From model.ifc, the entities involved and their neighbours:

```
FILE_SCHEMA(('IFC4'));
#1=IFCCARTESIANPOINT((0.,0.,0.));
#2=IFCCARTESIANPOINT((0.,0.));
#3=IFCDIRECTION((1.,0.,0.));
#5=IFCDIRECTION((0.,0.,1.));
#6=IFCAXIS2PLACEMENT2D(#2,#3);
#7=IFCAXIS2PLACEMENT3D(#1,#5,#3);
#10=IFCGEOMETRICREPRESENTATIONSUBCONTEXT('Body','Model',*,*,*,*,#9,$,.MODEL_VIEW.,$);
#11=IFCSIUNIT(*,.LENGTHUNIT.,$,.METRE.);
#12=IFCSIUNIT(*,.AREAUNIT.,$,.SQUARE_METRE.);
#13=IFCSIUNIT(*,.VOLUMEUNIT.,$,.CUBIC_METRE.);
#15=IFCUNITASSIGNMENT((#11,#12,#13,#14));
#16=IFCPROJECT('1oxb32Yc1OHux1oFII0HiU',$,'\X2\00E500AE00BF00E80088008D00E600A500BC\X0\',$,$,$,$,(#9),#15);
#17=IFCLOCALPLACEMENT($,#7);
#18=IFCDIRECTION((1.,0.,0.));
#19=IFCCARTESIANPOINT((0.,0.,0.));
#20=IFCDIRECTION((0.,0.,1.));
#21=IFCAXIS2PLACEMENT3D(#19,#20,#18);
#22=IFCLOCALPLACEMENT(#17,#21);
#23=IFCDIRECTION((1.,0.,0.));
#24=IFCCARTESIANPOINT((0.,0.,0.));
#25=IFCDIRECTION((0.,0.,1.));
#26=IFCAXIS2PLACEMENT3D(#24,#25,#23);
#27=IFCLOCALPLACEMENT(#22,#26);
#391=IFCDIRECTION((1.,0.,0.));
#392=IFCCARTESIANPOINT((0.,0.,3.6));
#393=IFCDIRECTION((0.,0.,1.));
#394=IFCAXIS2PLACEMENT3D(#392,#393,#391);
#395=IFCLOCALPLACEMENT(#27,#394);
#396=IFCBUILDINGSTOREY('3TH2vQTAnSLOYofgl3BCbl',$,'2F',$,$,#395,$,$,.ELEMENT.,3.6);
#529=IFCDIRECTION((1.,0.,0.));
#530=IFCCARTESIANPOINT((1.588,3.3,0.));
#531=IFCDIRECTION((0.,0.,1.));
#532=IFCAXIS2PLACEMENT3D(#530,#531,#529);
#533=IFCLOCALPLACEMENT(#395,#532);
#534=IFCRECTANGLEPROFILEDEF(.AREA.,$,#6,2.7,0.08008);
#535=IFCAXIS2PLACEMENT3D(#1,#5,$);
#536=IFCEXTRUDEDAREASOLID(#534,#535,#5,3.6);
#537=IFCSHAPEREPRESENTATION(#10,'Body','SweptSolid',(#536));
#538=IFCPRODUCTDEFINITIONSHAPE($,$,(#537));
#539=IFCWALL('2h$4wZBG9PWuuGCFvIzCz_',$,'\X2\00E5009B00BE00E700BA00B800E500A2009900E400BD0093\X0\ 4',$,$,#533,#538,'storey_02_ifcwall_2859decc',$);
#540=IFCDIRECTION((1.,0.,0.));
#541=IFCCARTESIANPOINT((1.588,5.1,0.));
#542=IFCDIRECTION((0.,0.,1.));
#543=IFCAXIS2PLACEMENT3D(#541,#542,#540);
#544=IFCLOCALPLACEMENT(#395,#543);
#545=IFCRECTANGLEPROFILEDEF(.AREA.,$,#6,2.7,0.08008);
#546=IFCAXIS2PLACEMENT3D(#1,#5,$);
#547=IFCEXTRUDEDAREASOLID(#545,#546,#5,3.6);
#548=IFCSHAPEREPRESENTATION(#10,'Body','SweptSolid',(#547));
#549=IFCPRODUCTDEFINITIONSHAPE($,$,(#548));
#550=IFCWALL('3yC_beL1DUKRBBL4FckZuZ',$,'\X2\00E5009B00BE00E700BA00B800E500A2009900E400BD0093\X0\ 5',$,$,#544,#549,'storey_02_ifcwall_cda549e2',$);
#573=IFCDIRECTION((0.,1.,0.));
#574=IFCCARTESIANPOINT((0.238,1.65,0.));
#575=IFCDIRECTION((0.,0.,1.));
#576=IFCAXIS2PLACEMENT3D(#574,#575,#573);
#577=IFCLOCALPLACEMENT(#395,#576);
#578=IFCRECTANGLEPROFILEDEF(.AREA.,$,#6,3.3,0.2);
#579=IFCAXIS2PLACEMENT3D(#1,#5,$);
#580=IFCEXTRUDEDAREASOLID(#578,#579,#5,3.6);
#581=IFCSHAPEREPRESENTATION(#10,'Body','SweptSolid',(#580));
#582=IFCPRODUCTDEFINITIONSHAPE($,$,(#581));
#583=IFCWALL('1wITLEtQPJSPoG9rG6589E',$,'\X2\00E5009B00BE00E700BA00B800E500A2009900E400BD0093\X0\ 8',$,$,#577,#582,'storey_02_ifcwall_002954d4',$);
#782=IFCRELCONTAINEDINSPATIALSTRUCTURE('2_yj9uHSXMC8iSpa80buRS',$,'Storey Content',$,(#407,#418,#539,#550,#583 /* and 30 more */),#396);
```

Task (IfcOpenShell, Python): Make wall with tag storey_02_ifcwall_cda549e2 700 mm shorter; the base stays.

```python
import ifcopenshell
import ifcopenshell.geom
import ifcopenshell.util.representation
import ifcopenshell.util.shape

model = ifcopenshell.open("model.ifc")
settings = ifcopenshell.geom.settings()


def volume(element):
    """Net volume in cubic metres, openings subtracted."""
    shape = ifcopenshell.geom.create_shape(settings, element)
    return ifcopenshell.util.shape.get_volume(shape.geometry)


wall = model.by_guid("3yC_beL1DUKRBBL4FckZuZ")
before = volume(wall)

body = ifcopenshell.util.representation.get_representation(wall, "Model", "Body")
solid = body.Items[0]
old_height = solid.Depth
solid.Depth -= 0.7
after = volume(wall)

print(f"height {old_height:g} -> {solid.Depth:g}, volume {before:.3f} -> {after:.3f} m3")

model.write("model_edited.ifc")
```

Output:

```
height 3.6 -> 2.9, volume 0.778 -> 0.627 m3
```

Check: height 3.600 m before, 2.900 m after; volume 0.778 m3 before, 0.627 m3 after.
